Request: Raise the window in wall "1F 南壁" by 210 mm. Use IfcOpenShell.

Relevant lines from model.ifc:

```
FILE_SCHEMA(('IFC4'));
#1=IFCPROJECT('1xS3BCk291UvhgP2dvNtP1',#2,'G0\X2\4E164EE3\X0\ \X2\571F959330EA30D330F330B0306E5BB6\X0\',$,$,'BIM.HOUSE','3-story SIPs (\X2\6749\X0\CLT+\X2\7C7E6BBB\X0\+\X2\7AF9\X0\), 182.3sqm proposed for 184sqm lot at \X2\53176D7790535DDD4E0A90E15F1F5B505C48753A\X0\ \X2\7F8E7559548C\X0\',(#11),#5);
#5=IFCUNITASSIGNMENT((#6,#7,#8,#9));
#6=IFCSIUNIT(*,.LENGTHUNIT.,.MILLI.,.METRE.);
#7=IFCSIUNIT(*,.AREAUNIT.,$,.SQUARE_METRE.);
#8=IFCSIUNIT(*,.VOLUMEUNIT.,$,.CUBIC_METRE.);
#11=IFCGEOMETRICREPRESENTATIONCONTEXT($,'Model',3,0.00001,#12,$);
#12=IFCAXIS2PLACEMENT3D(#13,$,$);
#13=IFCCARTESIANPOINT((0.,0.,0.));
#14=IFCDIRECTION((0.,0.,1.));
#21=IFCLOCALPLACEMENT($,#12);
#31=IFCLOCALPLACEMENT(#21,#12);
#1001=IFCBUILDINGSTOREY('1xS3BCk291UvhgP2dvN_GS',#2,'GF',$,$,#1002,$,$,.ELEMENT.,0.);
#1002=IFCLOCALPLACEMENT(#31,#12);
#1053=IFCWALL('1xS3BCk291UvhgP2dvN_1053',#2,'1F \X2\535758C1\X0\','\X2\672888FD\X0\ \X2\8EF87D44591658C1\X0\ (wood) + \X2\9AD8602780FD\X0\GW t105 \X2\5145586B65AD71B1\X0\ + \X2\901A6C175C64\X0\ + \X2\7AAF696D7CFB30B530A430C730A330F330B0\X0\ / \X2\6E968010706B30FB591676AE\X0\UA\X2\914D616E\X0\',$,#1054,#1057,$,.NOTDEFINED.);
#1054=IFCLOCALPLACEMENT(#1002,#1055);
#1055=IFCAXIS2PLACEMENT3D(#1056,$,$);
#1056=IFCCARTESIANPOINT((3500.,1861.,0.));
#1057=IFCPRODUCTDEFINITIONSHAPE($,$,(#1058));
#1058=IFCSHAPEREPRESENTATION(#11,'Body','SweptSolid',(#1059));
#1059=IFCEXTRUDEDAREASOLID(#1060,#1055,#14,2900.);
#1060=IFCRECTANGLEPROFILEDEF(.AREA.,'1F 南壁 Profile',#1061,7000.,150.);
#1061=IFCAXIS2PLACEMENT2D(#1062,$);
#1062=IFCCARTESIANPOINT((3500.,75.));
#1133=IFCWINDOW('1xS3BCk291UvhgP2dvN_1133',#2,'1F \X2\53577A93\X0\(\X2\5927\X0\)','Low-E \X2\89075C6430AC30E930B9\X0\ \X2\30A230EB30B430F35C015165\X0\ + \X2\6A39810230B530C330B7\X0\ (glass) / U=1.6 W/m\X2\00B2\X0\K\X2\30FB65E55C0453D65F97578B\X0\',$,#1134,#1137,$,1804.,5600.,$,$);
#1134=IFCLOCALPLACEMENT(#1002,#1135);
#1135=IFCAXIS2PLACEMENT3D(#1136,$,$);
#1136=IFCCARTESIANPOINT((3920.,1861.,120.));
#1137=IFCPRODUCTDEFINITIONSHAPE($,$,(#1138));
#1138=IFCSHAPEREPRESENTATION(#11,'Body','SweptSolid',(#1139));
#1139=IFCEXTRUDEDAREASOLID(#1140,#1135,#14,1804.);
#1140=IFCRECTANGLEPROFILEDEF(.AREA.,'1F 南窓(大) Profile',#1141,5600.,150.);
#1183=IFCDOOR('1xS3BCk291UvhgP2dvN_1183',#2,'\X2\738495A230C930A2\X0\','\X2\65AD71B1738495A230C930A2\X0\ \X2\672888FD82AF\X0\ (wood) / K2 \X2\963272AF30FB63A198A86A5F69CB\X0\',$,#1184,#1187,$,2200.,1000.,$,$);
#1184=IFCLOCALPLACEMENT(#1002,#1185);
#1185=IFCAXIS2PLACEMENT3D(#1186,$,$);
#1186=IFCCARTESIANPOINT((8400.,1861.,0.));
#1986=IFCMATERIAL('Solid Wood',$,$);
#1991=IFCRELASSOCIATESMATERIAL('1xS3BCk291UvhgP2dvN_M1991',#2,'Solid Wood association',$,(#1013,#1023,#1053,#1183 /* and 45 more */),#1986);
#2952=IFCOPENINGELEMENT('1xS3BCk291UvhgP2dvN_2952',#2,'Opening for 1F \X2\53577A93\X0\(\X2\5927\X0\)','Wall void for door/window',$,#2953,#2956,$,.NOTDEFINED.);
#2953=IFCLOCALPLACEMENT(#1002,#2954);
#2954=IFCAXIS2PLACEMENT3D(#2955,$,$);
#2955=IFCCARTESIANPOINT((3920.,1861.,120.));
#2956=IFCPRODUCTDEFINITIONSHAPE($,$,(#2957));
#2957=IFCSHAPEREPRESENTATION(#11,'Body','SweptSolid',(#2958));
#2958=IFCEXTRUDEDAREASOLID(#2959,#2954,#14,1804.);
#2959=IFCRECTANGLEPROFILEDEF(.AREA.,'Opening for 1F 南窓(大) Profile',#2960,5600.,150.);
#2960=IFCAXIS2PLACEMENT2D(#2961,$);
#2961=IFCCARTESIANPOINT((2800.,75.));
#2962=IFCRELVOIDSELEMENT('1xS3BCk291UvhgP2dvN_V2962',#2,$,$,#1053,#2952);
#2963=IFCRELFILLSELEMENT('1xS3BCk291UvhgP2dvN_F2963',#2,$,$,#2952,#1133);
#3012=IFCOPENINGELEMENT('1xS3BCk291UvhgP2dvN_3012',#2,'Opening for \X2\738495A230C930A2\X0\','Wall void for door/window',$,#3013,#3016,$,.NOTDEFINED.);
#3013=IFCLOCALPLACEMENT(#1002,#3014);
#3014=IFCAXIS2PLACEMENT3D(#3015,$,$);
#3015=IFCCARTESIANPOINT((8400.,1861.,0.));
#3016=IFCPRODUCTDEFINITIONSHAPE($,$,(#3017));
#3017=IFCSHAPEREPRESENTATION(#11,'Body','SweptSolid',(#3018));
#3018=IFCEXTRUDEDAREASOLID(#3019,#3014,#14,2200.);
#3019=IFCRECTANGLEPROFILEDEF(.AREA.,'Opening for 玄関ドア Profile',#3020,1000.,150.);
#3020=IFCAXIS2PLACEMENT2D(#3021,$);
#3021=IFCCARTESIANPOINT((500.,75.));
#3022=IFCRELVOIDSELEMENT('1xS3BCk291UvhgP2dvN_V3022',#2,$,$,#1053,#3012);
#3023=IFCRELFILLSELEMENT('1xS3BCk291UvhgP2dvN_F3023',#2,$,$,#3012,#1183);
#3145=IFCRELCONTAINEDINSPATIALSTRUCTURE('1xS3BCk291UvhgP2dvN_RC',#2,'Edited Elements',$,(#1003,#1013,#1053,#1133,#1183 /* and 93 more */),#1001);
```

```python
import numpy as np
import ifcopenshell
import ifcopenshell.api.geometry
import ifcopenshell.util.placement
import ifcopenshell.util.unit

model = ifcopenshell.open("model.ifc")
unit_scale = ifcopenshell.util.unit.calculate_unit_scale(model)

window = model.by_guid("1xS3BCk291UvhgP2dvN_1133")
opening = window.FillsVoids[0].RelatingOpeningElement
dz = 0.21 / unit_scale

shift = np.array([0.0, 0.0, dz])
# The window is not placed relative to its opening, so move both.
for product in (opening, window):
    matrix = ifcopenshell.util.placement.get_local_placement(product.ObjectPlacement)
    matrix[:3, 3] += shift
    ifcopenshell.api.geometry.edit_object_placement(model, product=product, matrix=matrix, is_si=False)

print(f"moved by {dz * unit_scale:+.3f} m")

model.write("model_updated.ifc")
```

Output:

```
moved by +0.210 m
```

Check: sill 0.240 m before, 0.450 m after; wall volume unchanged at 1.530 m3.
